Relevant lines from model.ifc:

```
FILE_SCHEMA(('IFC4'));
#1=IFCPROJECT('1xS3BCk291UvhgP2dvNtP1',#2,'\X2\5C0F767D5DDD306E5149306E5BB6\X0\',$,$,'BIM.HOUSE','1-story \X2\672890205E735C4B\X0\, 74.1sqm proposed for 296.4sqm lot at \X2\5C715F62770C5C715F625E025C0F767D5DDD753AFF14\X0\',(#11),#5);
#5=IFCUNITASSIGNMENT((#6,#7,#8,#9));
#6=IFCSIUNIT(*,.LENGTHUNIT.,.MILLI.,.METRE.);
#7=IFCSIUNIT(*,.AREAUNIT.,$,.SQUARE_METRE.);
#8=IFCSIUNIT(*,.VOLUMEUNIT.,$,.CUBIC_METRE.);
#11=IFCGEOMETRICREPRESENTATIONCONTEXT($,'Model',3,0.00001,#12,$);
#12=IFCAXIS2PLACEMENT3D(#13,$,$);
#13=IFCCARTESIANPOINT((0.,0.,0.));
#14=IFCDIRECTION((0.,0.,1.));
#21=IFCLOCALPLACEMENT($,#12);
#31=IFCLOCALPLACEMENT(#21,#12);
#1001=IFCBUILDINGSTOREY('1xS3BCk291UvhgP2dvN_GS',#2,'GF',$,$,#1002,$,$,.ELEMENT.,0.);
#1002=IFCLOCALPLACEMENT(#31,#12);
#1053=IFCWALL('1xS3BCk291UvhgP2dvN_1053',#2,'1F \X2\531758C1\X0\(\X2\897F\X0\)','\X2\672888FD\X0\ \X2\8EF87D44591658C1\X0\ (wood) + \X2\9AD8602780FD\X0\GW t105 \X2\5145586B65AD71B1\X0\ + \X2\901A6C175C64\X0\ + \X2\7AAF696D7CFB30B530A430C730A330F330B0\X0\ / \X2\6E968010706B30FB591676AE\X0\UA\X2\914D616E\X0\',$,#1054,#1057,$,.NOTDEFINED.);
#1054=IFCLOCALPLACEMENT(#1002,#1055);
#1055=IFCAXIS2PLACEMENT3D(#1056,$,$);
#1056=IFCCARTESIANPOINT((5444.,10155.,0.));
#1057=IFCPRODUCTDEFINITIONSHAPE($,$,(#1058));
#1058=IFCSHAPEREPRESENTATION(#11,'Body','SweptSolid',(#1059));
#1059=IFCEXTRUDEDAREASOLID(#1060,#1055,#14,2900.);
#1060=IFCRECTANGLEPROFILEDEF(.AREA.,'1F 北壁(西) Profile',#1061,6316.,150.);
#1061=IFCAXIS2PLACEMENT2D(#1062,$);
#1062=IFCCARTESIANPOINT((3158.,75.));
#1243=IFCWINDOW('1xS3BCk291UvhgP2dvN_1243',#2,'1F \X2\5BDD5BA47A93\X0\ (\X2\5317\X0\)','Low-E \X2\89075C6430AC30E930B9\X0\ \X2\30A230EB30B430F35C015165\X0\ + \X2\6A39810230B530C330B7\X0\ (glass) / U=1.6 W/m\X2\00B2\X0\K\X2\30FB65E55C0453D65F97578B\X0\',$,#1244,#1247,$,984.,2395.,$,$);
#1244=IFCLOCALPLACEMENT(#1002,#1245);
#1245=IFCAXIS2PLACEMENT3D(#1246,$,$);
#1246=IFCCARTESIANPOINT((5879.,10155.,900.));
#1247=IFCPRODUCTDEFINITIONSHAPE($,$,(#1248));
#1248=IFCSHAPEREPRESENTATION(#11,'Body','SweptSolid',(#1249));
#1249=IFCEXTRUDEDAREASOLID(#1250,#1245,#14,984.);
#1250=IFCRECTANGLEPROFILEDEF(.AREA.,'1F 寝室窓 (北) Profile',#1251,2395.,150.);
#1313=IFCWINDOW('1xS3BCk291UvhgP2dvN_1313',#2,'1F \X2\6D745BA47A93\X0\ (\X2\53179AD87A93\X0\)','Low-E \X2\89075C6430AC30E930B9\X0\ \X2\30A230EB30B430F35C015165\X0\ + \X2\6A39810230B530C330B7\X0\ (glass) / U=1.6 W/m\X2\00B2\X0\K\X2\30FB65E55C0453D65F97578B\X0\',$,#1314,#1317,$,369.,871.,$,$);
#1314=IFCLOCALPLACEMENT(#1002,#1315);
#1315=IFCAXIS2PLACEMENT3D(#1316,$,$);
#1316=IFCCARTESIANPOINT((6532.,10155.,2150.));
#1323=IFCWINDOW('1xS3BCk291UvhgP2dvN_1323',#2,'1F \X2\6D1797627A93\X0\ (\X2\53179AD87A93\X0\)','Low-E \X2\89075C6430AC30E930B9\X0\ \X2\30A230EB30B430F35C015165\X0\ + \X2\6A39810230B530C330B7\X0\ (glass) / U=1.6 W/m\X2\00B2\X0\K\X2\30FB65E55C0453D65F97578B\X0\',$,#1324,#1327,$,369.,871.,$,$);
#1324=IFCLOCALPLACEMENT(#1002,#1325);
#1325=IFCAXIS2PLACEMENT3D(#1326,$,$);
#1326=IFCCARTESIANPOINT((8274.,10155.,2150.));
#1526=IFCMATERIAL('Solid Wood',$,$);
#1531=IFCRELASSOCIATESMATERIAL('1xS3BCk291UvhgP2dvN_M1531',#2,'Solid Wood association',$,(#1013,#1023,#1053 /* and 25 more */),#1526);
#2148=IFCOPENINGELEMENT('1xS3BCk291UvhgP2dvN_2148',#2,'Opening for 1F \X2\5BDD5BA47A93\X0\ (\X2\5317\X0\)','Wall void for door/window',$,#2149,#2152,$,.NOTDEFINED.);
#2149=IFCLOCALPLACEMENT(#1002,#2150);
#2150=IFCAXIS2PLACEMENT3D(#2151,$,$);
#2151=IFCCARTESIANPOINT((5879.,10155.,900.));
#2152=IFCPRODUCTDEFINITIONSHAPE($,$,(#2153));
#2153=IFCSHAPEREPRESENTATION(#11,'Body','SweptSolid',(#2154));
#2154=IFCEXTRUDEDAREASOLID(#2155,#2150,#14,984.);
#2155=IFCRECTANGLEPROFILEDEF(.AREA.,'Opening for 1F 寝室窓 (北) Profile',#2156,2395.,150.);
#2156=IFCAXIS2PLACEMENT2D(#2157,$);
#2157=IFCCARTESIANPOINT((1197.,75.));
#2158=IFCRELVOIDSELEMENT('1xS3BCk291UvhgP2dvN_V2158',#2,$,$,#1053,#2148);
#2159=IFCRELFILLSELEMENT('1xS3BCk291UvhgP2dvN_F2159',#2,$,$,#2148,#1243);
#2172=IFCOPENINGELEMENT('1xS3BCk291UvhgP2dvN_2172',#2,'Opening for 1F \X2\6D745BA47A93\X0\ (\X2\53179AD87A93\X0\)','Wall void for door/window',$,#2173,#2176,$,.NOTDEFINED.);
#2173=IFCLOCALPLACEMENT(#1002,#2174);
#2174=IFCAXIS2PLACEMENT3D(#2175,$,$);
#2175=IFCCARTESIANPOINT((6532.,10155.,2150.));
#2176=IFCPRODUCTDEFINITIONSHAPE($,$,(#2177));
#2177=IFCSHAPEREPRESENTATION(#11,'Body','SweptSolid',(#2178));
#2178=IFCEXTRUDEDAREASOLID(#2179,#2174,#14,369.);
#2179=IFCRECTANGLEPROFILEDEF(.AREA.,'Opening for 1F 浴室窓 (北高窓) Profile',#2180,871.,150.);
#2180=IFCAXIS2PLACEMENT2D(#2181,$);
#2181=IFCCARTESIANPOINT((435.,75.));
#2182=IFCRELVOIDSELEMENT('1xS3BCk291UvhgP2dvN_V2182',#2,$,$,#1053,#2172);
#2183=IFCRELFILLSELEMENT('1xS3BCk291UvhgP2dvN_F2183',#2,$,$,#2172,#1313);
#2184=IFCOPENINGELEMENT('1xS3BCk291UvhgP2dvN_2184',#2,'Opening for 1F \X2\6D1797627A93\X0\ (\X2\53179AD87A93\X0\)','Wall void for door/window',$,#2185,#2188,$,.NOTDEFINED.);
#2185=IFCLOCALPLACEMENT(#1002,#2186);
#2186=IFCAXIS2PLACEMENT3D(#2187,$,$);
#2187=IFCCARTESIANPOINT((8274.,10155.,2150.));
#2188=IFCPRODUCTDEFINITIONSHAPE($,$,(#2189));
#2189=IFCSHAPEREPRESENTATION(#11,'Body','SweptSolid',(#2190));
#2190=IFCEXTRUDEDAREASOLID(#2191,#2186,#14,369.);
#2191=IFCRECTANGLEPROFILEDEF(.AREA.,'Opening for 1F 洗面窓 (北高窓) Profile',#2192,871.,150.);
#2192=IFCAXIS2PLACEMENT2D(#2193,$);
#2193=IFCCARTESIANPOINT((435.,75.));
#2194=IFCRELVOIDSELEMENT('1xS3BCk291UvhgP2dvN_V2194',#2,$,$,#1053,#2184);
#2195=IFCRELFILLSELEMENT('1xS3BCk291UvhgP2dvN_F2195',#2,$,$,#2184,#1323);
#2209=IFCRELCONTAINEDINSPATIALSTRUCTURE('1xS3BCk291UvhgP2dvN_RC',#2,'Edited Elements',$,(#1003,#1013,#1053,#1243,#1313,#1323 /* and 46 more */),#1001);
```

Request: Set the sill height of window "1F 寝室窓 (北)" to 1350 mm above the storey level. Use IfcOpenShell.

```python
import numpy as np
import ifcopenshell
import ifcopenshell.api.geometry
import ifcopenshell.geom
import ifcopenshell.util.element
import ifcopenshell.util.placement
import ifcopenshell.util.shape
import ifcopenshell.util.unit

model = ifcopenshell.open("model.ifc")
unit_scale = ifcopenshell.util.unit.calculate_unit_scale(model)

window = model.by_guid("1xS3BCk291UvhgP2dvN_1243")
opening = window.FillsVoids[0].RelatingOpeningElement
storey = ifcopenshell.util.element.get_container(window, ifc_class="IfcBuildingStorey")
level = ifcopenshell.util.placement.get_local_placement(storey.ObjectPlacement)[2, 3]

# The opening's origin need not be at the sill, so measure its lowest point.
shape = ifcopenshell.geom.create_shape(ifcopenshell.geom.settings(), opening)
bottom = ifcopenshell.util.shape.get_shape_bottom_elevation(shape, shape.geometry) / unit_scale
dz = level + 1350.0 - bottom

shift = np.array([0.0, 0.0, dz])
# The window is not placed relative to its opening, so move both.
for product in (opening, window):
    matrix = ifcopenshell.util.placement.get_local_placement(product.ObjectPlacement)
    matrix[:3, 3] += shift
    ifcopenshell.api.geometry.edit_object_placement(model, product=product, matrix=matrix, is_si=False)

print(f"moved by {dz * unit_scale:+.3f} m")

model.write("model_rev.ifc")
```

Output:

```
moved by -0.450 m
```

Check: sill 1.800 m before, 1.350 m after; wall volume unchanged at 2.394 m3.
